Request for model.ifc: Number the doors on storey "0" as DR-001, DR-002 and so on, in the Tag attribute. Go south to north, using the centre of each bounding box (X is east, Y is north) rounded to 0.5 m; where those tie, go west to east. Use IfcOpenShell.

First a look at what the model holds.

```python
import ifcopenshell
import ifcopenshell.util.element
import ifcopenshell.util.placement

model = ifcopenshell.open("model.ifc")
print(model.schema)
storey = next(s for s in model.by_type("IfcBuildingStorey") if s.Name == "0")
doors = [e for e in ifcopenshell.util.element.get_decomposition(storey) if e.is_a("IfcDoor")]
for e in sorted(doors, key=lambda e: e.id()):
    origin = ifcopenshell.util.placement.get_local_placement(e.ObjectPlacement)[:3, 3]
    print(e.id(), e.Tag, e.Name, origin.round(2) + 0.0, sep=" | ")
```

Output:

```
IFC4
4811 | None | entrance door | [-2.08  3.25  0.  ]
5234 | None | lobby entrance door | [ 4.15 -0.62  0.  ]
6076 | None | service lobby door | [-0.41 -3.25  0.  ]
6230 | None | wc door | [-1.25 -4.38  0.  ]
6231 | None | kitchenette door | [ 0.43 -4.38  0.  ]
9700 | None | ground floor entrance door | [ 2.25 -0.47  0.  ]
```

```python
import ifcopenshell
import ifcopenshell.geom
import ifcopenshell.util.element
import ifcopenshell.util.shape

model = ifcopenshell.open("model.ifc")
settings = ifcopenshell.geom.settings()
settings.set("use-world-coords", True)


def centre(element):
    shape = ifcopenshell.geom.create_shape(settings, element)
    return ifcopenshell.util.shape.get_bbox_centroid(shape.geometry)


storey = next(s for s in model.by_type("IfcBuildingStorey") if s.Name == "0")
doors = [e for e in ifcopenshell.util.element.get_decomposition(storey) if e.is_a("IfcDoor")]

# Insertion points can sit at a corner or the storey origin, so sort by the geometry (in metres).
centres = {e: centre(e) for e in doors}
doors.sort(key=lambda e: (round(centres[e][1] / 0.5), centres[e][0]))

for i, e in enumerate(doors, start=1):
    number = f"DR-0{i:02d}"
    e.Tag = number
    print(e.id(), number)

model.write("model_updated.ifc")
```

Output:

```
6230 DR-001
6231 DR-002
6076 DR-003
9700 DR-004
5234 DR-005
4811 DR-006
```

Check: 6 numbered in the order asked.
